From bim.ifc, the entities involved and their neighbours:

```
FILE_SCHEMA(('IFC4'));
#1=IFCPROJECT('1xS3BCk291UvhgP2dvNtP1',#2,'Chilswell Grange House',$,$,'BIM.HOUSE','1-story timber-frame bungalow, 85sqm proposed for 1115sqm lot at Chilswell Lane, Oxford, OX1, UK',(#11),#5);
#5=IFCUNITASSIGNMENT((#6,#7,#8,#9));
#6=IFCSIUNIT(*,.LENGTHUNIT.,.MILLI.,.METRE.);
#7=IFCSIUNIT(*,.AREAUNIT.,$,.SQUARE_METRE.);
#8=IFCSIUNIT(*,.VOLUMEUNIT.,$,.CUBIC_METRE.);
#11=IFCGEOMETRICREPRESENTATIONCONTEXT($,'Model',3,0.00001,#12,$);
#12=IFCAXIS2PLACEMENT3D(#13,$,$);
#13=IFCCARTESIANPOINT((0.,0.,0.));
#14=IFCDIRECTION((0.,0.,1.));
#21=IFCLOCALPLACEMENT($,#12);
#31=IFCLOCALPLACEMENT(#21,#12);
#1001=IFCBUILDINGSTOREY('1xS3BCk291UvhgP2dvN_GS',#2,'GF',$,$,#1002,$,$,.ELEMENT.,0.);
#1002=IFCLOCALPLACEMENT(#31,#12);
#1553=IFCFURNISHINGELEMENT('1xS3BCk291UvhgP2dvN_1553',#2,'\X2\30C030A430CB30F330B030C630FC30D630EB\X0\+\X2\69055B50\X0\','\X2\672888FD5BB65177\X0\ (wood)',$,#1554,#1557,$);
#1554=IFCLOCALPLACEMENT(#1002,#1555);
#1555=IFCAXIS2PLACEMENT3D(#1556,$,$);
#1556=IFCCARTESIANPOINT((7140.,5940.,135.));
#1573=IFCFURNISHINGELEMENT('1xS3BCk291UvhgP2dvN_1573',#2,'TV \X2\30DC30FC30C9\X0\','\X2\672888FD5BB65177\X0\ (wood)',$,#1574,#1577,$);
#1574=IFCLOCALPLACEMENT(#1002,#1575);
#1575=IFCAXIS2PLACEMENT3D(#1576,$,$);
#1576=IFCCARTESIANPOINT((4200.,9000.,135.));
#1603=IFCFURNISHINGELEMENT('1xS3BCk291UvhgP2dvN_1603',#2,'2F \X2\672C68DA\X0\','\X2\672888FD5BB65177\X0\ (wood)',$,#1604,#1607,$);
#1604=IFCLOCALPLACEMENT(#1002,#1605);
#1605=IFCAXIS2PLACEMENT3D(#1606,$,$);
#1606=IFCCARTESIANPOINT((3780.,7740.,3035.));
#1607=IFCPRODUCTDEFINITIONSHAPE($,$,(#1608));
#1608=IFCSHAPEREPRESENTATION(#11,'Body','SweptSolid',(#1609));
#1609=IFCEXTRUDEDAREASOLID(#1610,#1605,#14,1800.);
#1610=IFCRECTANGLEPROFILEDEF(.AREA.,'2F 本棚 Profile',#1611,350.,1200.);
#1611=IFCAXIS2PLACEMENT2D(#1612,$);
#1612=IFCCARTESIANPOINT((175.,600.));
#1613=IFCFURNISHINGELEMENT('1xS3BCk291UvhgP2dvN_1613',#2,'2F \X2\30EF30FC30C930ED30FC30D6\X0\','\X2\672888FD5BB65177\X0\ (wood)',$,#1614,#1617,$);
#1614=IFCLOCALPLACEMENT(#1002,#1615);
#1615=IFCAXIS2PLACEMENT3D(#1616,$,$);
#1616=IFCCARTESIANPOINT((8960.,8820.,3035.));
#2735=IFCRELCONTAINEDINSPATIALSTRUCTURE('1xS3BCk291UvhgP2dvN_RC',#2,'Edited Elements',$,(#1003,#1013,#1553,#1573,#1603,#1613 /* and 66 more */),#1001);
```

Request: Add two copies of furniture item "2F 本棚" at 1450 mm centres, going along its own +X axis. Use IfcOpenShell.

```python
import ifcopenshell
import ifcopenshell.api.geometry
import ifcopenshell.api.root
import ifcopenshell.util.element
import ifcopenshell.util.placement

model = ifcopenshell.open("bim.ifc")


def reuse_history(source, copy):
    """copy_class also copies each property set's owner history, people and application; keep the originals."""
    for rel in copy.IsDefinedBy:
        if rel.is_a("IfcRelDefinesByProperties") and (history := rel.RelatingPropertyDefinition.OwnerHistory):
            rel.RelatingPropertyDefinition.OwnerHistory = source.OwnerHistory
            ifcopenshell.util.element.remove_deep2(model, history)


source = model.by_guid("1xS3BCk291UvhgP2dvN_1603")
base = ifcopenshell.util.placement.get_local_placement(source.ObjectPlacement)
step = base[:3, 0] * 1450.0

for i in range(1, 3):
    copy = ifcopenshell.api.root.copy_class(model, product=source)
    copy.Representation = ifcopenshell.util.element.copy_deep(
        model, source.Representation, exclude=["IfcGeometricRepresentationContext", "IfcRepresentationMap"]
    )
    reuse_history(source, copy)
    matrix = base.copy()
    matrix[:3, 3] += i * step
    print("added at", matrix[:3, 3].round(3) + 0.0)
    ifcopenshell.api.geometry.edit_object_placement(model, product=copy, matrix=matrix, is_si=False)

model.write("bim_rev.ifc")
```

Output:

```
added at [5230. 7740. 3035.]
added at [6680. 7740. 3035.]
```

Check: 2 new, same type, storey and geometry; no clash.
